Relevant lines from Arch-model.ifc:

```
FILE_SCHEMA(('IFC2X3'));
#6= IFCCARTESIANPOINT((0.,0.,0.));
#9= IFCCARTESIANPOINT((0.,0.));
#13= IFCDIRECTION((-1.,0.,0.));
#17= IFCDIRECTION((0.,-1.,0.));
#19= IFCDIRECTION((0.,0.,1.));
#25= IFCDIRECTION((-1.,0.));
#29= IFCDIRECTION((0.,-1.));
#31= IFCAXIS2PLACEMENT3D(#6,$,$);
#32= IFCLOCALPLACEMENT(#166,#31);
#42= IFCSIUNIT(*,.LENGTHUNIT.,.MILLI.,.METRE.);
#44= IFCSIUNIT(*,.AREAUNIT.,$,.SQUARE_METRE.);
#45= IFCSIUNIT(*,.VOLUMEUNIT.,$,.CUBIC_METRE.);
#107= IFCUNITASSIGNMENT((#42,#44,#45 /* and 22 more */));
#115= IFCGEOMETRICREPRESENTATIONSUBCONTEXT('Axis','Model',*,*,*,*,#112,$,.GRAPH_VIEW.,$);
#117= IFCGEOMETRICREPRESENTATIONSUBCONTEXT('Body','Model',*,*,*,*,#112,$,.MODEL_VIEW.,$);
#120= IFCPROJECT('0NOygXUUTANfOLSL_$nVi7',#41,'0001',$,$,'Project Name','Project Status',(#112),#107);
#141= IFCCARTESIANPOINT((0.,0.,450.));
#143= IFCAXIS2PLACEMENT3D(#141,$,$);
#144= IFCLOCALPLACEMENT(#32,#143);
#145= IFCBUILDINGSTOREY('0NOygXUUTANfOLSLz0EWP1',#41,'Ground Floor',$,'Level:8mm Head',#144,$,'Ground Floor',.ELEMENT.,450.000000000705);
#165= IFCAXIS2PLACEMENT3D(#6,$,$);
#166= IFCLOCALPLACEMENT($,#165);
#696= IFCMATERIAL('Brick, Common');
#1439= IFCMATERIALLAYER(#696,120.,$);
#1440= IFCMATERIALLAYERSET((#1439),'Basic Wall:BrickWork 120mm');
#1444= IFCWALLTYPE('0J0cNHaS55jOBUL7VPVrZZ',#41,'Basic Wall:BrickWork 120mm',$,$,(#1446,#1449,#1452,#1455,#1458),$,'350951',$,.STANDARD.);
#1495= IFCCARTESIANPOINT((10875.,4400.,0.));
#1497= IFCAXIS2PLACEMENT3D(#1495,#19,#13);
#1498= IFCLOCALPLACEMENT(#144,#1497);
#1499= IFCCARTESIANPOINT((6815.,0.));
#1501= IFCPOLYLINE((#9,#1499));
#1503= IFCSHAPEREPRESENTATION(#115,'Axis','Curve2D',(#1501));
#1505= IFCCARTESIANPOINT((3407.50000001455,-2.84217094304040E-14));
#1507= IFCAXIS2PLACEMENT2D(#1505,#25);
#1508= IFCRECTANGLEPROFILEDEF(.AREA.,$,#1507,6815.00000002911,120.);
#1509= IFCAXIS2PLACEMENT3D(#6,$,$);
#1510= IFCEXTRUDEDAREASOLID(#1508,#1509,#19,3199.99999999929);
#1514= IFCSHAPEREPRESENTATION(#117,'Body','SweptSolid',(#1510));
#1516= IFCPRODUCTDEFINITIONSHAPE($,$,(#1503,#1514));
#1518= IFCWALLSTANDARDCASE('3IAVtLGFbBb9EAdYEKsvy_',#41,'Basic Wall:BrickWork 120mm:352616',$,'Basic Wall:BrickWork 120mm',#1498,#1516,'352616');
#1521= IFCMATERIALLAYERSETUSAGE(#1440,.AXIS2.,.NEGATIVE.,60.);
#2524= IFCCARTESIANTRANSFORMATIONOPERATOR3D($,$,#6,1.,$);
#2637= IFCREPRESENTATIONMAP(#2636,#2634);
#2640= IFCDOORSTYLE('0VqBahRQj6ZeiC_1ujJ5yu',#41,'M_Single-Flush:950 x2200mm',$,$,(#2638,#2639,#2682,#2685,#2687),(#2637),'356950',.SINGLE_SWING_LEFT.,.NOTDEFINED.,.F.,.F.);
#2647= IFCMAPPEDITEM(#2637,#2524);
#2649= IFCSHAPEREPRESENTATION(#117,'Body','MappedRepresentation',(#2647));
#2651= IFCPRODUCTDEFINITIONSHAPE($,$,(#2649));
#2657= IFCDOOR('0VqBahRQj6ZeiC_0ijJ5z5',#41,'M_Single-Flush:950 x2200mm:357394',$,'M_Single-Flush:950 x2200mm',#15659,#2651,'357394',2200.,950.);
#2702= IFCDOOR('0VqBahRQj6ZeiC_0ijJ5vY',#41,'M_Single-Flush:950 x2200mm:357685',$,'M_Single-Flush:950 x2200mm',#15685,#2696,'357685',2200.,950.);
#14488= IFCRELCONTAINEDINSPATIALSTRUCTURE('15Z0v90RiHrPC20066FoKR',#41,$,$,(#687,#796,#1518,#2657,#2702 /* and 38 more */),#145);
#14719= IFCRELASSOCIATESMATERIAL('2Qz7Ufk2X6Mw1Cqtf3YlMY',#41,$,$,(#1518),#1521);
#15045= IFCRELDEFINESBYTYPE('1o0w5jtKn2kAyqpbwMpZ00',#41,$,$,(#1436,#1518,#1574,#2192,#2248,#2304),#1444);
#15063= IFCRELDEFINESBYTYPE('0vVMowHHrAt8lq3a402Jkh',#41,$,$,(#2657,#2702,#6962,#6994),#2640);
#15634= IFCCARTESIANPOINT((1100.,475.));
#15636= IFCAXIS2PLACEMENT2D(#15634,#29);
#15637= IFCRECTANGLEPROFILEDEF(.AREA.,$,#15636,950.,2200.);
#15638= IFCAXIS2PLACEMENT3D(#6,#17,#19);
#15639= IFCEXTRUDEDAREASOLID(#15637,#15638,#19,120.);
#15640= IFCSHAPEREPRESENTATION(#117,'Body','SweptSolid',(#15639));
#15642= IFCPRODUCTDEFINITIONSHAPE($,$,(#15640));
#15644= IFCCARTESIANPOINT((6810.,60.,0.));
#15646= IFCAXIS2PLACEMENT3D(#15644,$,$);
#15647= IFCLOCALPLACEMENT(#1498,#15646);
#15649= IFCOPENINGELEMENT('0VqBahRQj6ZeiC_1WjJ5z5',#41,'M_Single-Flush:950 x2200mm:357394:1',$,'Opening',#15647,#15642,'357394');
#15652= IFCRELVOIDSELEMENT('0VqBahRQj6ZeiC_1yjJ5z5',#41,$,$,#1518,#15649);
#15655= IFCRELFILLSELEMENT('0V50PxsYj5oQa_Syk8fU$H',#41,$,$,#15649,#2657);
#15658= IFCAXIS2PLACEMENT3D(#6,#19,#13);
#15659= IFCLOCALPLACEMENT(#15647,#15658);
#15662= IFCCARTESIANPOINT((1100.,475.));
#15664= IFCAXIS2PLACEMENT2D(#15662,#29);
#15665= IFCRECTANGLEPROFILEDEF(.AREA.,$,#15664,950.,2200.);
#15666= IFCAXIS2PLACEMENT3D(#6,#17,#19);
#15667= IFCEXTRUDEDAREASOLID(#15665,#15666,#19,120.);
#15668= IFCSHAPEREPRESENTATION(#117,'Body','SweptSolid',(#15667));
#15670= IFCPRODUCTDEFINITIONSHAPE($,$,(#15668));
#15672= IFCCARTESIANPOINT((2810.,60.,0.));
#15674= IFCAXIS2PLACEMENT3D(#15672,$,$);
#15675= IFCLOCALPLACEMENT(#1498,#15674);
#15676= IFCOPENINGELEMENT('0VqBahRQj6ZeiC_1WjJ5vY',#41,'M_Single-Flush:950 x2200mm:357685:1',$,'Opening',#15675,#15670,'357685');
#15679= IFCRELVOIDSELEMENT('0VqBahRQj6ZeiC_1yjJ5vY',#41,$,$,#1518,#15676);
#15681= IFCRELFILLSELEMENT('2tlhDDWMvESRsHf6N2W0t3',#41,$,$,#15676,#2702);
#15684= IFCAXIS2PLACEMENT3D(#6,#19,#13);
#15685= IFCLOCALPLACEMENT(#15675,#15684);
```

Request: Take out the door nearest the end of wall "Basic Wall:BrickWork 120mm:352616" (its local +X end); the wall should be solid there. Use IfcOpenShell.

```python
import ifcopenshell
import ifcopenshell.api.feature
import ifcopenshell.api.root
import ifcopenshell.geom
import ifcopenshell.util.shape

model = ifcopenshell.open("Arch-model.ifc")
settings = ifcopenshell.geom.settings()


def volume(element):
    """Net volume in cubic metres, openings subtracted."""
    shape = ifcopenshell.geom.create_shape(settings, element)
    return ifcopenshell.util.shape.get_volume(shape.geometry)


door = model.by_guid("0VqBahRQj6ZeiC_0ijJ5z5")
opening = door.FillsVoids[0].RelatingOpeningElement
wall = opening.VoidsElements[0].RelatingBuildingElement
before = volume(wall)

ifcopenshell.api.root.remove_product(model, product=door)
ifcopenshell.api.feature.remove_feature(model, feature=opening)

after = volume(wall)

print(f"wall volume {before:.3f} -> {after:.3f} m3")

model.write("Arch-model-out.ifc")
```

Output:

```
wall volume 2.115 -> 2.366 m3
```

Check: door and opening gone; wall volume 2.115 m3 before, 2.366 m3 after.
